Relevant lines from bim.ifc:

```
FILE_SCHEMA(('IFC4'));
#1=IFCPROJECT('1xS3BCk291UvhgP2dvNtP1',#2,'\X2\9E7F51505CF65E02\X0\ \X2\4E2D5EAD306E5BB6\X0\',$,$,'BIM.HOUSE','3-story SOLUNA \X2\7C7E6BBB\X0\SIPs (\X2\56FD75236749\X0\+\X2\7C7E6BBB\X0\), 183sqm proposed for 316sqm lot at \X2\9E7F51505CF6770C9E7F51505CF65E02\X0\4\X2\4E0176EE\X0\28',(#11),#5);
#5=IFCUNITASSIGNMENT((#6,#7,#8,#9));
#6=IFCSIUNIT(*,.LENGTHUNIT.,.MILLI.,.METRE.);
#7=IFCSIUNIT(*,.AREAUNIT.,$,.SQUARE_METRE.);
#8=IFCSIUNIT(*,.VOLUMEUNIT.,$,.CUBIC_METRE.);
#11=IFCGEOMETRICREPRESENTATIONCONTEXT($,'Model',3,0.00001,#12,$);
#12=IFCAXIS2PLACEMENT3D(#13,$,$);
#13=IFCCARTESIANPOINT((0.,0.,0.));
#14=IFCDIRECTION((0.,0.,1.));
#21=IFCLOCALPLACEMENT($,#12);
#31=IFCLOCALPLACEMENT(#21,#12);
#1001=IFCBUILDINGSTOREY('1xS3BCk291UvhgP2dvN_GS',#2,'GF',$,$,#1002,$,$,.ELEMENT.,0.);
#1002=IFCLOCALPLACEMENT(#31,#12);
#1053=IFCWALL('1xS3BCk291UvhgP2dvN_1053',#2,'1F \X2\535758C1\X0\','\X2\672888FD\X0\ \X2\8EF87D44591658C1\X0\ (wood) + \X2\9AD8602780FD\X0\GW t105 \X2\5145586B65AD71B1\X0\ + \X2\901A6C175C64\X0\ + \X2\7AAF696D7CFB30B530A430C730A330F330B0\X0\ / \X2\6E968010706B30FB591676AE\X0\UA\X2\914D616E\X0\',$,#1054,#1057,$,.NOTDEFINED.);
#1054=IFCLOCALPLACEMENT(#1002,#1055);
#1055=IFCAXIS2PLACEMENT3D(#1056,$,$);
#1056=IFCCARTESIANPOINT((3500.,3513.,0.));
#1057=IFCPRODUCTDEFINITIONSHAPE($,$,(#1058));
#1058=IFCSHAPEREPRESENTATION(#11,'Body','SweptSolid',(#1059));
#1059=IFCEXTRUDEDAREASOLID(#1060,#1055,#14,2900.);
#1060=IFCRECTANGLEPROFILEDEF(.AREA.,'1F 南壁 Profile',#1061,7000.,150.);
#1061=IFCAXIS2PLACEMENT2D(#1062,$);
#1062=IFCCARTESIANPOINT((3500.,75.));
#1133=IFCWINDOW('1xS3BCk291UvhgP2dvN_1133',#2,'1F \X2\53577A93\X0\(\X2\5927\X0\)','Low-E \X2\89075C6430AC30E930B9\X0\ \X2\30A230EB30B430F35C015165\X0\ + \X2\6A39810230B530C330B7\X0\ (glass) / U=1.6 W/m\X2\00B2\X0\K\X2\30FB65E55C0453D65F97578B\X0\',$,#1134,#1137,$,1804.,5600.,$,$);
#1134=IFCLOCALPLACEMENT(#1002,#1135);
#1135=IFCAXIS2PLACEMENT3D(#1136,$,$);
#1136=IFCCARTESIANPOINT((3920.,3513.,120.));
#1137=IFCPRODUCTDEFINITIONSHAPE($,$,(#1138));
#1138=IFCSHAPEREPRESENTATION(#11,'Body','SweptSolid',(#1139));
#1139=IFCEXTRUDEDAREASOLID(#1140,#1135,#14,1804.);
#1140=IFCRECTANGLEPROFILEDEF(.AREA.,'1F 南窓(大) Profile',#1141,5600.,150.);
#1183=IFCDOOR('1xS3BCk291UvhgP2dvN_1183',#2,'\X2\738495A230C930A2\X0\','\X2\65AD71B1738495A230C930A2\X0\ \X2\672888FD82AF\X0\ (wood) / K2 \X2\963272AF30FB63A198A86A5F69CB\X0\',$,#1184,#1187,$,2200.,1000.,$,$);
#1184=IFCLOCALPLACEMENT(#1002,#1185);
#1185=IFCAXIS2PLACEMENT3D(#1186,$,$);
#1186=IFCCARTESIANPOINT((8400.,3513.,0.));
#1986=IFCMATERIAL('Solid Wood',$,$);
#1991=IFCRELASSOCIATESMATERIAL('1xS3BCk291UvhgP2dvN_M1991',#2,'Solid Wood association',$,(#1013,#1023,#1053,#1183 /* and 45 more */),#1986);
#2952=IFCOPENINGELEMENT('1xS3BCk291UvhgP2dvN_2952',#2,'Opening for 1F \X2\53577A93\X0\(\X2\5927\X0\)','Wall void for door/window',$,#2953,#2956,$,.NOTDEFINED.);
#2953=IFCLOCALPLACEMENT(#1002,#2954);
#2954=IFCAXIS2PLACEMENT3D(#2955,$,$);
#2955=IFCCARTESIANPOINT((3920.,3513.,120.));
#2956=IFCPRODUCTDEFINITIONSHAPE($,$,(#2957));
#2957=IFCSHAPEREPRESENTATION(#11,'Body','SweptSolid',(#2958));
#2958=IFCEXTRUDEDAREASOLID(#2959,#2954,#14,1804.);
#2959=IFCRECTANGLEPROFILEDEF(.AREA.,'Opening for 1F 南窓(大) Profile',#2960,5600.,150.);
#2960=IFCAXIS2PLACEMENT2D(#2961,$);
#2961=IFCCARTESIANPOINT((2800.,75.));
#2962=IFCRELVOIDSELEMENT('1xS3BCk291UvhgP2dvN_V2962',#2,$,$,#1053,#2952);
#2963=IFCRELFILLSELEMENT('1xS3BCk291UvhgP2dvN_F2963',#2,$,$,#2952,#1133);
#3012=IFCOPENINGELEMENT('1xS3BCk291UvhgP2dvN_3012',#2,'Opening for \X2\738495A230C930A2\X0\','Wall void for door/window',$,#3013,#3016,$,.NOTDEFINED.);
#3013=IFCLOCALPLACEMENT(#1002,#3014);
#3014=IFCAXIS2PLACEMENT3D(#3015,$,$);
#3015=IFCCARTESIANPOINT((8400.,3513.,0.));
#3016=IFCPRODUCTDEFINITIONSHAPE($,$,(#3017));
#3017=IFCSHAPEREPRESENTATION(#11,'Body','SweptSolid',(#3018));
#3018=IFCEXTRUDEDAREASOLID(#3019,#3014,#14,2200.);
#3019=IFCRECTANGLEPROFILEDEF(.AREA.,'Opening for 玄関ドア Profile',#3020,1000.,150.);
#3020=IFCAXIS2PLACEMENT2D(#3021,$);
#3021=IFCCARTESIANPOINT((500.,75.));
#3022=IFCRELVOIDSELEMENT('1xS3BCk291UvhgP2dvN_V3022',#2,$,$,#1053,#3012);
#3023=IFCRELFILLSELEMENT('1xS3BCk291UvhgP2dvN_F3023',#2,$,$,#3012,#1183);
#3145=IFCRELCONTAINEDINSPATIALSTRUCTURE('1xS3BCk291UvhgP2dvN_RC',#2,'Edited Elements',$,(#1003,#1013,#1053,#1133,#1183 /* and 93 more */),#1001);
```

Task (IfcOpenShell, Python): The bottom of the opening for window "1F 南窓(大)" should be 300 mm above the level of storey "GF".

```python
import numpy as np
import ifcopenshell
import ifcopenshell.api.geometry
import ifcopenshell.geom
import ifcopenshell.util.element
import ifcopenshell.util.placement
import ifcopenshell.util.shape
import ifcopenshell.util.unit

model = ifcopenshell.open("bim.ifc")
unit_scale = ifcopenshell.util.unit.calculate_unit_scale(model)

window = model.by_id(1133)
opening = window.FillsVoids[0].RelatingOpeningElement
storey = ifcopenshell.util.element.get_container(window, ifc_class="IfcBuildingStorey")
level = ifcopenshell.util.placement.get_local_placement(storey.ObjectPlacement)[2, 3]

# The opening's origin need not be at the sill, so measure its lowest point.
shape = ifcopenshell.geom.create_shape(ifcopenshell.geom.settings(), opening)
bottom = ifcopenshell.util.shape.get_shape_bottom_elevation(shape, shape.geometry) / unit_scale
dz = level + 0.3 / unit_scale - bottom

shift = np.array([0.0, 0.0, dz])
# The window is not placed relative to its opening, so move both.
for product in (opening, window):
    matrix = ifcopenshell.util.placement.get_local_placement(product.ObjectPlacement)
    matrix[:3, 3] += shift
    ifcopenshell.api.geometry.edit_object_placement(model, product=product, matrix=matrix, is_si=False)

print(f"moved by {dz * unit_scale:+.3f} m")

model.write("bim_updated.ifc")
```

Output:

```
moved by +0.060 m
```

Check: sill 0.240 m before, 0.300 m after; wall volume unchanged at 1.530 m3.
